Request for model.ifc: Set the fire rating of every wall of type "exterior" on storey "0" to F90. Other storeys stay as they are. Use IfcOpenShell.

First a look at what the model holds.

```python
import ifcopenshell
import ifcopenshell.util.element

model = ifcopenshell.open("model.ifc")
print(model.schema)
storey = next(s for s in model.by_type("IfcBuildingStorey") if s.Name == "0")
walls = [e for e in ifcopenshell.util.element.get_decomposition(storey) if e.is_a("IfcWall")]
seen = {}
for e in walls:
    element_type = ifcopenshell.util.element.get_type(e)
    key = (element_type.Name if element_type != e and element_type else None, ifcopenshell.util.element.get_pset(e, "Pset_WallCommon", "FireRating"))
    seen[key] = seen.get(key, 0) + 1
for (name, value), count in sorted(seen.items(), key=str):
    print(count, "x", name, "|", value)
```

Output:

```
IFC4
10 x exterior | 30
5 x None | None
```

```python
import ifcopenshell
import ifcopenshell.api.pset
import ifcopenshell.util.element

model = ifcopenshell.open("model.ifc")

storey = next(s for s in model.by_type("IfcBuildingStorey") if s.Name == "0")
walls = [e for e in ifcopenshell.util.element.get_decomposition(storey) if e.is_a("IfcWall")]

count = 0
for e in walls:
    element_type = ifcopenshell.util.element.get_type(e)
    if element_type in (None, e) or element_type.Name != "exterior":
        continue
    # add_pset returns the element's existing set when there is one.
    pset = ifcopenshell.api.pset.add_pset(model, product=e, name="Pset_WallCommon")
    ifcopenshell.api.pset.edit_pset(model, pset=pset, properties={"FireRating": "F90"})
    count += 1

print(count, "walls updated")

model.write("model_edited.ifc")
```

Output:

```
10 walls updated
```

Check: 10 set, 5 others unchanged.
